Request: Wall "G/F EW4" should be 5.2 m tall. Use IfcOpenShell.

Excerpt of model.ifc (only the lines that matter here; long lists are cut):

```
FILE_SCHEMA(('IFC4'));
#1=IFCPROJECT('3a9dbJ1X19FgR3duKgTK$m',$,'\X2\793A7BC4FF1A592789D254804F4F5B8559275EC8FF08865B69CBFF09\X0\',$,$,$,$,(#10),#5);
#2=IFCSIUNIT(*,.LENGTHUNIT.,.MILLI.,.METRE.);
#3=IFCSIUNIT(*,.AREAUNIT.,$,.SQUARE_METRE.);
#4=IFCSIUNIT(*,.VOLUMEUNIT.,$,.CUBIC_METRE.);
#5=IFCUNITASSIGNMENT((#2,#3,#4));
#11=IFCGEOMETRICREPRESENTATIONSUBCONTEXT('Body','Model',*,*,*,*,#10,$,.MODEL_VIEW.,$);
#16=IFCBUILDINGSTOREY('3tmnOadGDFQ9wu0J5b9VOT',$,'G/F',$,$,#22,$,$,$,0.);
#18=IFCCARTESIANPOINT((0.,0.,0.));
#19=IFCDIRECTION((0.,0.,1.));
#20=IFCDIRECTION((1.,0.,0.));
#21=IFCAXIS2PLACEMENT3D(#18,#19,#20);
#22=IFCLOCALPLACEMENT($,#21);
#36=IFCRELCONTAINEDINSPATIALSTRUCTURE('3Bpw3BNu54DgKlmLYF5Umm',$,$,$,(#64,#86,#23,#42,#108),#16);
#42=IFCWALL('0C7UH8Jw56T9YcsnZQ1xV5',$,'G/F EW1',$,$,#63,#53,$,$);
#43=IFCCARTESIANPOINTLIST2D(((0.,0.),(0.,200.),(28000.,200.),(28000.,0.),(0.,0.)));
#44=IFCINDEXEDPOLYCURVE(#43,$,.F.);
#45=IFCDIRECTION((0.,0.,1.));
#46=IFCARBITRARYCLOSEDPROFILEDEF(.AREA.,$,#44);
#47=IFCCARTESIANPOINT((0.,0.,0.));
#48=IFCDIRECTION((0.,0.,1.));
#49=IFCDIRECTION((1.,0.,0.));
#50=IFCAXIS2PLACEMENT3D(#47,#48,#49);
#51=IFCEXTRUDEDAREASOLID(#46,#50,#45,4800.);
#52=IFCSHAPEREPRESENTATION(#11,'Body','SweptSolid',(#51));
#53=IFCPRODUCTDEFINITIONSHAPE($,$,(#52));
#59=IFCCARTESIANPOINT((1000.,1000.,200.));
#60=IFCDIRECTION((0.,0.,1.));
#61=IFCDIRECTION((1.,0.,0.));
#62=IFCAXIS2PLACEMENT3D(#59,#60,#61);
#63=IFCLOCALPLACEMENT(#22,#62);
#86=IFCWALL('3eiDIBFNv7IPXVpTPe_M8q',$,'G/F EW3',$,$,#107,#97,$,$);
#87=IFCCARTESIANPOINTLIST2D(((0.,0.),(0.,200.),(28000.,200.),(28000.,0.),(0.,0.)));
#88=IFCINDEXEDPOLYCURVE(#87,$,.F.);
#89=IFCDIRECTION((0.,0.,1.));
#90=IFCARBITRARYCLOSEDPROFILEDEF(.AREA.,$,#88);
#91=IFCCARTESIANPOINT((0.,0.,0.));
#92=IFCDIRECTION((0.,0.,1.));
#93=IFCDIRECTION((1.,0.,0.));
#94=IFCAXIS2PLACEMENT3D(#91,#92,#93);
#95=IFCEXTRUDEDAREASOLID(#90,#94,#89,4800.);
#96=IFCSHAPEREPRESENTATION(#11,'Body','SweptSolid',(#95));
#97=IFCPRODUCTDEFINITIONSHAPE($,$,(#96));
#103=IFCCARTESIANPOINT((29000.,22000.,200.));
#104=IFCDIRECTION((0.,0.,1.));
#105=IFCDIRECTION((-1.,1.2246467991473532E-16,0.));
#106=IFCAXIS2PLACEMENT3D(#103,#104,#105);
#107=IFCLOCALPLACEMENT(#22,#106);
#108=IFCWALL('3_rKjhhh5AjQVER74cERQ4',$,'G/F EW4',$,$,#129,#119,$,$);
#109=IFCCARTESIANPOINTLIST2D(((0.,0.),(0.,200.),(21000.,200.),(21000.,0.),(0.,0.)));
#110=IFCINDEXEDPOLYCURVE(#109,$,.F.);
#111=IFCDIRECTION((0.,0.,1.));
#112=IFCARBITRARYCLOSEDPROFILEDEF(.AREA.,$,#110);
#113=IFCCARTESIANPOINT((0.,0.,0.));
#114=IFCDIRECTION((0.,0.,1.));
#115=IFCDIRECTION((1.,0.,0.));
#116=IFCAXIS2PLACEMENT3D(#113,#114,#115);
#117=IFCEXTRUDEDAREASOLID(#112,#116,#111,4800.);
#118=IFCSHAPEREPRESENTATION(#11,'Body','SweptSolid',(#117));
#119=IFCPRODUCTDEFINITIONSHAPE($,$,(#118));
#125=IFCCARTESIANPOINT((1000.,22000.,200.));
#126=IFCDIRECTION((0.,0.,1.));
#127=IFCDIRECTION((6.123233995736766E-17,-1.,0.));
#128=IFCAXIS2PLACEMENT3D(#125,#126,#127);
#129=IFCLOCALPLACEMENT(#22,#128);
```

```python
import ifcopenshell
import ifcopenshell.geom
import ifcopenshell.util.representation
import ifcopenshell.util.shape
import ifcopenshell.util.unit

model = ifcopenshell.open("model.ifc")
unit_scale = ifcopenshell.util.unit.calculate_unit_scale(model)
settings = ifcopenshell.geom.settings()


def volume(element):
    """Net volume in cubic metres, openings subtracted."""
    shape = ifcopenshell.geom.create_shape(settings, element)
    return ifcopenshell.util.shape.get_volume(shape.geometry)


wall = model.by_guid("3_rKjhhh5AjQVER74cERQ4")
before = volume(wall)

body = ifcopenshell.util.representation.get_representation(wall, "Model", "Body")
solid = body.Items[0]
old_height = solid.Depth
solid.Depth = 5.2 / unit_scale
after = volume(wall)

print(f"height {old_height:g} -> {solid.Depth:g}, volume {before:.3f} -> {after:.3f} m3")

model.write("model-out.ifc")
```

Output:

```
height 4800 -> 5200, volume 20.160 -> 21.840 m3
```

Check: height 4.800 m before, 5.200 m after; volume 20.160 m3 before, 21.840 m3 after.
